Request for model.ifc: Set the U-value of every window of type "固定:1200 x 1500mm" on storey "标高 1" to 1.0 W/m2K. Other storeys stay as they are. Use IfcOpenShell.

First a look at what the model holds.

```python
import ifcopenshell
import ifcopenshell.util.element

model = ifcopenshell.open("model.ifc")
print(model.schema)
storey = next(s for s in model.by_type("IfcBuildingStorey") if s.Name == "标高 1")
windows = [e for e in ifcopenshell.util.element.get_decomposition(storey) if e.is_a("IfcWindow")]
seen = {}
for e in windows:
    element_type = ifcopenshell.util.element.get_type(e)
    key = (element_type.Name if element_type != e and element_type else None, ifcopenshell.util.element.get_pset(e, "Pset_WindowCommon", "ThermalTransmittance"))
    seen[key] = seen.get(key, 0) + 1
for (name, value), count in sorted(seen.items(), key=str):
    print(count, "x", name, "|", value)
```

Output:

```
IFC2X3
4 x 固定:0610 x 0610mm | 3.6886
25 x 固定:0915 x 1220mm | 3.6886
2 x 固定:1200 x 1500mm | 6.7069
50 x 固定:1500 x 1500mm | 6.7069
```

```python
import ifcopenshell
import ifcopenshell.api.pset
import ifcopenshell.util.element

model = ifcopenshell.open("model.ifc")

storey = next(s for s in model.by_type("IfcBuildingStorey") if s.Name == "标高 1")
windows = [e for e in ifcopenshell.util.element.get_decomposition(storey) if e.is_a("IfcWindow")]

count = 0
for e in windows:
    element_type = ifcopenshell.util.element.get_type(e)
    if element_type in (None, e) or element_type.Name != "固定:1200 x 1500mm":
        continue
    # add_pset returns the element's existing set when there is one.
    pset = ifcopenshell.api.pset.add_pset(model, product=e, name="Pset_WindowCommon")
    ifcopenshell.api.pset.edit_pset(model, pset=pset, properties={"ThermalTransmittance": 1.0})
    count += 1

print(count, "windows updated")

model.write("model_edited.ifc")
```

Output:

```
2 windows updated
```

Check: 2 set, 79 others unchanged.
